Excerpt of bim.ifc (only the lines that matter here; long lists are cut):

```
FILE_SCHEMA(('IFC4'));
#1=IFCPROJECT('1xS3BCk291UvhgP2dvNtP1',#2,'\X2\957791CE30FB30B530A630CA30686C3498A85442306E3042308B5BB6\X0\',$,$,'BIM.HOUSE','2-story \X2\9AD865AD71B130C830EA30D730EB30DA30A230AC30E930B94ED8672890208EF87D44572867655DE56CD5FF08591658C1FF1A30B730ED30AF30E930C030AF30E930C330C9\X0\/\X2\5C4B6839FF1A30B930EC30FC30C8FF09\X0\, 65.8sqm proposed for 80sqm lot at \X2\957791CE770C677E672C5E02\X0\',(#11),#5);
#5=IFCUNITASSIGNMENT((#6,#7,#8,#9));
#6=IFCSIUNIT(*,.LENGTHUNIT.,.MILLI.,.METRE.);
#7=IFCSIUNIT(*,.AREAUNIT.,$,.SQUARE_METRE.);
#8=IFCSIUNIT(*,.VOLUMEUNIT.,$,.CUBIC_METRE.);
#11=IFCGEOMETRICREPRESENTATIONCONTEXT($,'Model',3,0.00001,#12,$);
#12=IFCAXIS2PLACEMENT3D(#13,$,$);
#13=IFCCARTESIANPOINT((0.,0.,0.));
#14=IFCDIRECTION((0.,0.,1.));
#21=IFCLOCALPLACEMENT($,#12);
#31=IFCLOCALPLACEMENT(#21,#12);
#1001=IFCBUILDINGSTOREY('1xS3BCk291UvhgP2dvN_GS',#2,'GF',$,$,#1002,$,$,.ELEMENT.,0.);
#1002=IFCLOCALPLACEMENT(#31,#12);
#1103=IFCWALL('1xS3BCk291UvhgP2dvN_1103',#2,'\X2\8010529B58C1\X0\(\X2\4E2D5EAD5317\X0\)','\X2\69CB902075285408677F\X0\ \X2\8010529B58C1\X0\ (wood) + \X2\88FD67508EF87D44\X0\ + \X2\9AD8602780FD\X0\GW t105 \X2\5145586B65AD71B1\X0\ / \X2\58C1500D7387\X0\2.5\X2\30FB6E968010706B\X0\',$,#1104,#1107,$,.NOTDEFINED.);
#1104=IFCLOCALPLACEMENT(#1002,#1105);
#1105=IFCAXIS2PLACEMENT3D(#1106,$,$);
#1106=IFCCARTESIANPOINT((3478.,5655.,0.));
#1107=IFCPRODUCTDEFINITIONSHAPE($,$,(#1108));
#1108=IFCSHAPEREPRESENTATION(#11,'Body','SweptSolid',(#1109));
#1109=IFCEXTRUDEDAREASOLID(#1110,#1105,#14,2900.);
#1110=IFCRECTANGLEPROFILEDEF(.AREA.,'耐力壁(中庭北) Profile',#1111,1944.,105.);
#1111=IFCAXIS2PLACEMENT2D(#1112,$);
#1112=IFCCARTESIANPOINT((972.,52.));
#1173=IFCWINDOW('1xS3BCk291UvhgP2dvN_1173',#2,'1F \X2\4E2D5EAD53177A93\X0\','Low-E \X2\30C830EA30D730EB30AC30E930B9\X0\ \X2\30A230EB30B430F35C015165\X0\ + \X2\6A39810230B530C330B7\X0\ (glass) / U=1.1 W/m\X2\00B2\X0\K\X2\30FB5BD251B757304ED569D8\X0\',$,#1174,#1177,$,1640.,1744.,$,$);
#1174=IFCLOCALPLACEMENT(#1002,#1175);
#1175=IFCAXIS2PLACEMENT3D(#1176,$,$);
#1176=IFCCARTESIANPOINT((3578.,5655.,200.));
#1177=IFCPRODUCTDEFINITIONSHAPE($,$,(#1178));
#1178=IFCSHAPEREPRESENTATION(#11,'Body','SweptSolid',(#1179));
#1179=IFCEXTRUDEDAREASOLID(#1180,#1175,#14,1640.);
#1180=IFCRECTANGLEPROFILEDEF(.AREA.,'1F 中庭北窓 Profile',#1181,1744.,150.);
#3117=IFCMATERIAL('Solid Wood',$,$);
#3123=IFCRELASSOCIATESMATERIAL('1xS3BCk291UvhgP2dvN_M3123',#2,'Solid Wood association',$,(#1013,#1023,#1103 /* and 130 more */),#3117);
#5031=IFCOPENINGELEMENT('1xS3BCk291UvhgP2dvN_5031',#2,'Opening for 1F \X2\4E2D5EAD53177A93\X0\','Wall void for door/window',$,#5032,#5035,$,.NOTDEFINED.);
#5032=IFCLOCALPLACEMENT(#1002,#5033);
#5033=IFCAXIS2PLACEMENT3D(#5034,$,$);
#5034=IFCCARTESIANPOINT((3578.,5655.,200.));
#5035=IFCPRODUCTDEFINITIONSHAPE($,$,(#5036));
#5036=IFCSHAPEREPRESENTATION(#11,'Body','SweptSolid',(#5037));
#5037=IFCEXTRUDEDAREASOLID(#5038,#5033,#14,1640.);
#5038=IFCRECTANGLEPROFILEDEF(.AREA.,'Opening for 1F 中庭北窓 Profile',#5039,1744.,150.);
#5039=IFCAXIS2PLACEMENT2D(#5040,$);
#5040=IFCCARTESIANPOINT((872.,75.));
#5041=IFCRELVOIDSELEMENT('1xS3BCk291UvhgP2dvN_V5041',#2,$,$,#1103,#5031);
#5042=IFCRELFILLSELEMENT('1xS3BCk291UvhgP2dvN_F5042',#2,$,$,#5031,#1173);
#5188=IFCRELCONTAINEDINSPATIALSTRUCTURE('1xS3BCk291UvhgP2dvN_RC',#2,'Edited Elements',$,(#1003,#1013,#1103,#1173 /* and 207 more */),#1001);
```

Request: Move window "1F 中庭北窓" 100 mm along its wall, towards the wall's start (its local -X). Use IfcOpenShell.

```python
import ifcopenshell
import ifcopenshell.api.geometry
import ifcopenshell.util.placement

model = ifcopenshell.open("bim.ifc")

window = model.by_guid("1xS3BCk291UvhgP2dvN_1173")
opening = window.FillsVoids[0].RelatingOpeningElement
wall = opening.VoidsElements[0].RelatingBuildingElement

wall_matrix = ifcopenshell.util.placement.get_local_placement(wall.ObjectPlacement)
shift = wall_matrix[:3, 0] * -100.0
before = ifcopenshell.util.placement.get_local_placement(window.ObjectPlacement)[:3, 3].copy()

# The window is not placed relative to its opening, so move both.
for product in (opening, window):
    matrix = ifcopenshell.util.placement.get_local_placement(product.ObjectPlacement)
    matrix[:3, 3] += shift
    ifcopenshell.api.geometry.edit_object_placement(model, product=product, matrix=matrix, is_si=False)

after = ifcopenshell.util.placement.get_local_placement(window.ObjectPlacement)[:3, 3]
print("window moved by", (after - before).round(3) + 0.0)

model.write("bim_rev.ifc")
```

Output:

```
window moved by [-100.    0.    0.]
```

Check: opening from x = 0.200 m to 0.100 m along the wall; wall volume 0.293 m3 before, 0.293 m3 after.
